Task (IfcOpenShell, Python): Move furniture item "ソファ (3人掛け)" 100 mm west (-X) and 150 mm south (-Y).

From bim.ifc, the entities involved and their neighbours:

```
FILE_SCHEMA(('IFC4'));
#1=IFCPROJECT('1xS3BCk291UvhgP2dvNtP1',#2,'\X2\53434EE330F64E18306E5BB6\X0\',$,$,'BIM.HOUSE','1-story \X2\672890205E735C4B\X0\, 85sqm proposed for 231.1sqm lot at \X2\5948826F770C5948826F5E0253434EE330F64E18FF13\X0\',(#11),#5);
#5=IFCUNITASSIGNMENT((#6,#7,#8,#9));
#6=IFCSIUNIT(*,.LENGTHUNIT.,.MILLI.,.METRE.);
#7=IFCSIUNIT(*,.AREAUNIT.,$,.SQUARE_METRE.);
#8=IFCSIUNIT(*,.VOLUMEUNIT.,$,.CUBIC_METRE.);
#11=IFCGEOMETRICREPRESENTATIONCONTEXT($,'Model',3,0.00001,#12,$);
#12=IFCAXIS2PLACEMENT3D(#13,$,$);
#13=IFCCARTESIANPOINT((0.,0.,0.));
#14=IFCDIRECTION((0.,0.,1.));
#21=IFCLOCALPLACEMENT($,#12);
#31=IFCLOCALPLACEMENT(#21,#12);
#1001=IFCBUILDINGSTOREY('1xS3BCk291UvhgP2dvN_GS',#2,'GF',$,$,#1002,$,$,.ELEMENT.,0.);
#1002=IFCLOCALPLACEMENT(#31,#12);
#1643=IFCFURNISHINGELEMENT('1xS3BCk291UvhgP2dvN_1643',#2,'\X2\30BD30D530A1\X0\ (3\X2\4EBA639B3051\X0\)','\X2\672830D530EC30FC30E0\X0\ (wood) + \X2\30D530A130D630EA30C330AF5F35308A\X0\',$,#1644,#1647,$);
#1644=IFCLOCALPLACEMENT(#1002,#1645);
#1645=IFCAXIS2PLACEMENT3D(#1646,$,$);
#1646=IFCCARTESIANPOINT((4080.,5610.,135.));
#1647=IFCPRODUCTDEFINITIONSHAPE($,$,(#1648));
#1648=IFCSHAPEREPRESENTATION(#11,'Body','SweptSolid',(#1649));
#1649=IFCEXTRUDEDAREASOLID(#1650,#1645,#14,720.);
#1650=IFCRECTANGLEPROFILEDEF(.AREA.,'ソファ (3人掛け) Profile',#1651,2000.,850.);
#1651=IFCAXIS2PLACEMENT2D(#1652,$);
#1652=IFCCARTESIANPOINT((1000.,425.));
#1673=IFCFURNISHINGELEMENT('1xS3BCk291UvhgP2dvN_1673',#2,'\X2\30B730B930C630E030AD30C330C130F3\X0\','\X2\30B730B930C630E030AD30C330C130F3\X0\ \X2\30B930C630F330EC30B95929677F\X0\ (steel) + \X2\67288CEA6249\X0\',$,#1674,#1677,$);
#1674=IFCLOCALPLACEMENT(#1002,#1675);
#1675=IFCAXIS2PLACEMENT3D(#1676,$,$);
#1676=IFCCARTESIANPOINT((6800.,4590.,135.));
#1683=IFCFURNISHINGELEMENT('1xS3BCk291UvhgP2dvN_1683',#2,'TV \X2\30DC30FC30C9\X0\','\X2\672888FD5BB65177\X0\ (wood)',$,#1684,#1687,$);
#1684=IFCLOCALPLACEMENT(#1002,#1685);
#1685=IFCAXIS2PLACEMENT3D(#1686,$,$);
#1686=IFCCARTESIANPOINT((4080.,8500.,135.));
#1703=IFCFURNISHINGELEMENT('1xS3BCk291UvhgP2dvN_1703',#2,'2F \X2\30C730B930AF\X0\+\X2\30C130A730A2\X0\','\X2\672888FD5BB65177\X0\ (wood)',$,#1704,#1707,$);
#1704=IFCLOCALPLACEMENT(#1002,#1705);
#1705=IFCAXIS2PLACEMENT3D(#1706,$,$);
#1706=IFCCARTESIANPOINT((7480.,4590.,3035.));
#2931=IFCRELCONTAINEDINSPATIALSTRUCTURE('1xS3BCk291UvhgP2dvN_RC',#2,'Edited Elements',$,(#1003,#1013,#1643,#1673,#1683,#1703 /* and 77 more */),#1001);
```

```python
import ifcopenshell
import ifcopenshell.api.geometry
import ifcopenshell.util.placement
import ifcopenshell.util.unit

model = ifcopenshell.open("bim.ifc")
unit_scale = ifcopenshell.util.unit.calculate_unit_scale(model)

item = model.by_guid("1xS3BCk291UvhgP2dvN_1643")
matrix = ifcopenshell.util.placement.get_local_placement(item.ObjectPlacement)
matrix[0, 3] -= 0.1 / unit_scale
matrix[1, 3] -= 0.15 / unit_scale
ifcopenshell.api.geometry.edit_object_placement(model, product=item, matrix=matrix, is_si=False)

print(ifcopenshell.util.placement.get_local_placement(item.ObjectPlacement).round(3) + 0.0)

model.write("bim_updated.ifc")
```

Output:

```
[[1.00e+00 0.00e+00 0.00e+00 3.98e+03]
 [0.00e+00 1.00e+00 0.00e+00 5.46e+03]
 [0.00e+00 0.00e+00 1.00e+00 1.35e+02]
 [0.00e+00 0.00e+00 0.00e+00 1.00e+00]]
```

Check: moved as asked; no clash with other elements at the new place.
